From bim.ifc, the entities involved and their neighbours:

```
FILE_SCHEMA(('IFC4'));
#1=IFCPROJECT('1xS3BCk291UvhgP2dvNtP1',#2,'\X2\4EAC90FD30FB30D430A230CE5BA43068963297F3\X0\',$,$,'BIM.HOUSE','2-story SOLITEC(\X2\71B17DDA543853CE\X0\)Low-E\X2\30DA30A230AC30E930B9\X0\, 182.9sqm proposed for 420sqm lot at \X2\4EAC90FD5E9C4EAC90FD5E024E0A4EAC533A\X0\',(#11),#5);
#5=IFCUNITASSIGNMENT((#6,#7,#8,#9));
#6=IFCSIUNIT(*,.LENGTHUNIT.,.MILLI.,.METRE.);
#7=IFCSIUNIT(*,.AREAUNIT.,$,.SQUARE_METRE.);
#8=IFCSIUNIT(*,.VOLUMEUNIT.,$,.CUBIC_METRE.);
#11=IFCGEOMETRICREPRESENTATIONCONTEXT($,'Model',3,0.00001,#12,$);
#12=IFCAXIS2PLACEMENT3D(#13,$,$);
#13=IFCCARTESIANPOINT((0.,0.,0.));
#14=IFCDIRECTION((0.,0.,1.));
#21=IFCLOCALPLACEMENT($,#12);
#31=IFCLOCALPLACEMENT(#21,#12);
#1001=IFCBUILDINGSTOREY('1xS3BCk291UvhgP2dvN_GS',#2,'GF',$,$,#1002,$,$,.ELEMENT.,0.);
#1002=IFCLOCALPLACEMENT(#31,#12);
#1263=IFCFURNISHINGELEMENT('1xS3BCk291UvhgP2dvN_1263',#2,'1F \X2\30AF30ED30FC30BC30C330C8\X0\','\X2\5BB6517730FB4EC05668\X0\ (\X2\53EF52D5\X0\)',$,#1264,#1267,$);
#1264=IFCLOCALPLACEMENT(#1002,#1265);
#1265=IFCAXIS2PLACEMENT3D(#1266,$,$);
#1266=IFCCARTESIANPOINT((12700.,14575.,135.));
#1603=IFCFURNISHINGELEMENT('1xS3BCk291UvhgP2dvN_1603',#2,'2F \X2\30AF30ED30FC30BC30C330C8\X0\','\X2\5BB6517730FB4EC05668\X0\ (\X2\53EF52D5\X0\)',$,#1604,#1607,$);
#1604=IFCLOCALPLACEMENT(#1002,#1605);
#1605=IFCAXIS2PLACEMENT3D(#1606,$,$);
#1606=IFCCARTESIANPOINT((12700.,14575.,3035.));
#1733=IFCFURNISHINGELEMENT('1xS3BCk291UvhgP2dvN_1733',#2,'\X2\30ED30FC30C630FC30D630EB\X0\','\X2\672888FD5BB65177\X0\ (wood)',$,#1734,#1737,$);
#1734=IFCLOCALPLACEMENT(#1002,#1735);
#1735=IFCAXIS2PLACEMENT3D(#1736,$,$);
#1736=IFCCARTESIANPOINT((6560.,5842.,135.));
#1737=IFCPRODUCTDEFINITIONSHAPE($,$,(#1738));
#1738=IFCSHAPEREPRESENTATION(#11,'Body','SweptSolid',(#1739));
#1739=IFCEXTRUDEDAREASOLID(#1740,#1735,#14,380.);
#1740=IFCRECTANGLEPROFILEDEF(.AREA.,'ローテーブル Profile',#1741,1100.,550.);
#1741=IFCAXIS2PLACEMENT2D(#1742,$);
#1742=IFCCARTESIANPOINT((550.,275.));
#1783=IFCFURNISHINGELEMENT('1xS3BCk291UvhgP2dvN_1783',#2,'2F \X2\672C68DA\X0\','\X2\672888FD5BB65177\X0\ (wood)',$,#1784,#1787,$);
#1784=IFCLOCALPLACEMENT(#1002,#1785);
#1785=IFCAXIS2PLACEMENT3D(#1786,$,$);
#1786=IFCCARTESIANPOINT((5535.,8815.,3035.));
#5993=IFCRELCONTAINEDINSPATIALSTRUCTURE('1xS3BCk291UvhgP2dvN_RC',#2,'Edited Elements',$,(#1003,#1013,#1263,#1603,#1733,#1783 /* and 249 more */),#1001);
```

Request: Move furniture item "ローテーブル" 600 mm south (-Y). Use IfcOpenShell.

```python
import ifcopenshell
import ifcopenshell.api.geometry
import ifcopenshell.util.placement
import ifcopenshell.util.unit

model = ifcopenshell.open("bim.ifc")
unit_scale = ifcopenshell.util.unit.calculate_unit_scale(model)

item = model.by_id(1733)
matrix = ifcopenshell.util.placement.get_local_placement(item.ObjectPlacement)
matrix[1, 3] -= 0.6 / unit_scale
ifcopenshell.api.geometry.edit_object_placement(model, product=item, matrix=matrix, is_si=False)

print(ifcopenshell.util.placement.get_local_placement(item.ObjectPlacement).round(3) + 0.0)

model.write("bim_updated.ifc")
```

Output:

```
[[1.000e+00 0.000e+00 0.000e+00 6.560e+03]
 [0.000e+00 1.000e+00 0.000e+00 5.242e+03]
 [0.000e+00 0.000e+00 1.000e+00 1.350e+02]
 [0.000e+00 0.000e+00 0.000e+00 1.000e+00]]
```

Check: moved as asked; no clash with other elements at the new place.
